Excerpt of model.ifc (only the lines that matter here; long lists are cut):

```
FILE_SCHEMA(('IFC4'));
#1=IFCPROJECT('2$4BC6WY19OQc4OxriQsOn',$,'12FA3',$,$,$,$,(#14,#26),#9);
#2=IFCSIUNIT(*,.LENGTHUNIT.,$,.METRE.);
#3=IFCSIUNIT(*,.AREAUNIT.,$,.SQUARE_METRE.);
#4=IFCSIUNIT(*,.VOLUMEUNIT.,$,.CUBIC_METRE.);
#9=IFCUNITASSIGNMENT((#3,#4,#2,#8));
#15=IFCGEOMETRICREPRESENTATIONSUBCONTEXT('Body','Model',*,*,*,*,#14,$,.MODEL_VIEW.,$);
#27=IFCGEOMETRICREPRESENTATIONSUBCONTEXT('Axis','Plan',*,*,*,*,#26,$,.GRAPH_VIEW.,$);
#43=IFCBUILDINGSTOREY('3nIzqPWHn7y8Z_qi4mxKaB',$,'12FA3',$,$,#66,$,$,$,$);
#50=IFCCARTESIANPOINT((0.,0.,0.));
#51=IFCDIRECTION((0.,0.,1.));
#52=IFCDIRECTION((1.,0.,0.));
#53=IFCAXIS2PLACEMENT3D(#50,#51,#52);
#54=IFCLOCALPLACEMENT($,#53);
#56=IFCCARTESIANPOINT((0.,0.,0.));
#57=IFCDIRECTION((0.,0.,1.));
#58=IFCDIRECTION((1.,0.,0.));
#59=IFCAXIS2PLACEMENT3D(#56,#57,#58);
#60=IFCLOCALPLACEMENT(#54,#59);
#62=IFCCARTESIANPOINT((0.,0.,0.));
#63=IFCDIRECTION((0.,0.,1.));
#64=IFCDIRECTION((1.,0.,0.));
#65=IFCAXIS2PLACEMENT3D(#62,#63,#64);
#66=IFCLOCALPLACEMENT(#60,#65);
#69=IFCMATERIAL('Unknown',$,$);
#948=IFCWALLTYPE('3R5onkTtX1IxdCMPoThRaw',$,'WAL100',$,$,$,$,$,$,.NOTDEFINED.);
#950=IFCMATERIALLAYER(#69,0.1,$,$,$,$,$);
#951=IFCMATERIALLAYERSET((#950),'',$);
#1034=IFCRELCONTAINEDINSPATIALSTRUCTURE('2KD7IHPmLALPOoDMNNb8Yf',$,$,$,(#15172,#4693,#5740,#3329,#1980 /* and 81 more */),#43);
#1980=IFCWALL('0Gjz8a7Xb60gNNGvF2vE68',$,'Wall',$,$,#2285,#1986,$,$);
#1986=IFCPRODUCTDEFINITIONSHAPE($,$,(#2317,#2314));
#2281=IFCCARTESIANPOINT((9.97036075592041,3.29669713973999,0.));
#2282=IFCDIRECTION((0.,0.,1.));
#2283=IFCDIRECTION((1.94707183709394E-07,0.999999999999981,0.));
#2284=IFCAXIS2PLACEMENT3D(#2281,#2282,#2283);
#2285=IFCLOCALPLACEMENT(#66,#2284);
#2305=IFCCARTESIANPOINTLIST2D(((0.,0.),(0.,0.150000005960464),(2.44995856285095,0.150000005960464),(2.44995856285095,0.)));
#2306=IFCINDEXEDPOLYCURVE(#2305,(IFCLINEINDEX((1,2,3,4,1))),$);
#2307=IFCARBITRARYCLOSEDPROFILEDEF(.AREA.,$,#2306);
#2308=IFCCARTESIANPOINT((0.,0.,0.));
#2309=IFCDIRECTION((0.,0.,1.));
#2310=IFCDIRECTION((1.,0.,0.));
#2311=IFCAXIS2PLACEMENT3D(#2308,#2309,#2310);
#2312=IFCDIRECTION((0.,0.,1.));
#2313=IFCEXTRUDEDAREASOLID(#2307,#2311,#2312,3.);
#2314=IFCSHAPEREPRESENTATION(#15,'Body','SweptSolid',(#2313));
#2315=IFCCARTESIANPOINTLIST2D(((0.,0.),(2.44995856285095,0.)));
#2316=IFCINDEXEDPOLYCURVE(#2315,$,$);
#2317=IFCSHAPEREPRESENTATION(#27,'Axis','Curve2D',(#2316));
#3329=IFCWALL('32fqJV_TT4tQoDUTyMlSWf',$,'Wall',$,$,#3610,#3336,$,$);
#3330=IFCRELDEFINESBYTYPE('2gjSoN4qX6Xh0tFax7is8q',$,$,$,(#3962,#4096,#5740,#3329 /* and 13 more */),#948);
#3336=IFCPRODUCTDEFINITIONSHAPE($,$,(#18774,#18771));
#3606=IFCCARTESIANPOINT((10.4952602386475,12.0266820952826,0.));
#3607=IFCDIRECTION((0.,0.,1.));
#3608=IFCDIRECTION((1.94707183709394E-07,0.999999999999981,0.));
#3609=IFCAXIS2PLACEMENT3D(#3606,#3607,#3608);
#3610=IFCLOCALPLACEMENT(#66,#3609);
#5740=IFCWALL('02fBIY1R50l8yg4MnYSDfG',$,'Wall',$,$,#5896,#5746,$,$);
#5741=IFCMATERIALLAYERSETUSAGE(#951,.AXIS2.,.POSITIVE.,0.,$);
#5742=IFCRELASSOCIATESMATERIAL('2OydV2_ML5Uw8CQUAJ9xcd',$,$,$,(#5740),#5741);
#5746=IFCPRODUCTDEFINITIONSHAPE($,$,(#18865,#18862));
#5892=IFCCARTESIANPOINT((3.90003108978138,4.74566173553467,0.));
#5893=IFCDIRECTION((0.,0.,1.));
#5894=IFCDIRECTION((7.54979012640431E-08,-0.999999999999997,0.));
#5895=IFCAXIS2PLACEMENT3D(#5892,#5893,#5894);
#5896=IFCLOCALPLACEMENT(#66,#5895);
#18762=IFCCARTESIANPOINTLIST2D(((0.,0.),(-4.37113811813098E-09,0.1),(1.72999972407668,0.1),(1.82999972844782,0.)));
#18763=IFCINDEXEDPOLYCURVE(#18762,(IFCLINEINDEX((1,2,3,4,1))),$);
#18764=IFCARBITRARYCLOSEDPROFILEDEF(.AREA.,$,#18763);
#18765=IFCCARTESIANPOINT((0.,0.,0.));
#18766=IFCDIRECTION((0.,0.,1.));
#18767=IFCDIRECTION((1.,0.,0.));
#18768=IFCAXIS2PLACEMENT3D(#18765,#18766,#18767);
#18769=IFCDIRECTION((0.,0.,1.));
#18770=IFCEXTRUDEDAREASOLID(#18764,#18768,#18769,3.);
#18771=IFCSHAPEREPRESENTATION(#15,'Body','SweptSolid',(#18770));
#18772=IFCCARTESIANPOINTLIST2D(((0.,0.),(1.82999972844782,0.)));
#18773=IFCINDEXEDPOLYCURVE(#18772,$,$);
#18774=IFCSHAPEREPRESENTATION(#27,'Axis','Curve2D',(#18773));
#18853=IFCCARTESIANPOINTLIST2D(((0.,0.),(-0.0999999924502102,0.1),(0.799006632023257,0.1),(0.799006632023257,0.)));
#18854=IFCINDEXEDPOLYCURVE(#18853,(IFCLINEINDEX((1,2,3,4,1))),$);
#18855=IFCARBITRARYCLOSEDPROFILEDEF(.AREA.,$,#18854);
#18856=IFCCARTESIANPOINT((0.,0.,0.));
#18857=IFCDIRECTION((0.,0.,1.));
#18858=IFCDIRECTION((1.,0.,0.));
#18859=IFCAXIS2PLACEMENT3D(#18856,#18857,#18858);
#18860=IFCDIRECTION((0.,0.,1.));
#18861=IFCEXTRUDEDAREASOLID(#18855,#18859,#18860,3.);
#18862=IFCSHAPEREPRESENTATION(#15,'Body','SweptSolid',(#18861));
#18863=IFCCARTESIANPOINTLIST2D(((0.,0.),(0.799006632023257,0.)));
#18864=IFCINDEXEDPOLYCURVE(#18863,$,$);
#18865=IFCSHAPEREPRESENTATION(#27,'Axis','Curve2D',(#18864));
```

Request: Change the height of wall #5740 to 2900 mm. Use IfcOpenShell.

```python
import ifcopenshell
import ifcopenshell.geom
import ifcopenshell.util.representation
import ifcopenshell.util.shape

model = ifcopenshell.open("model.ifc")
settings = ifcopenshell.geom.settings()


def volume(element):
    """Net volume in cubic metres, openings subtracted."""
    shape = ifcopenshell.geom.create_shape(settings, element)
    return ifcopenshell.util.shape.get_volume(shape.geometry)


wall = model.by_guid("02fBIY1R50l8yg4MnYSDfG")
before = volume(wall)

body = ifcopenshell.util.representation.get_representation(wall, "Model", "Body")
solid = body.Items[0]
old_height = solid.Depth
solid.Depth = 2.9
after = volume(wall)

print(f"height {old_height:g} -> {solid.Depth:g}, volume {before:.3f} -> {after:.3f} m3")

model.write("model_v2.ifc")
```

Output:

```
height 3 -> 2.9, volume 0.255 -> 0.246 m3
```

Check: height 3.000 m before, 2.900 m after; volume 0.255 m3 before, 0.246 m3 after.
